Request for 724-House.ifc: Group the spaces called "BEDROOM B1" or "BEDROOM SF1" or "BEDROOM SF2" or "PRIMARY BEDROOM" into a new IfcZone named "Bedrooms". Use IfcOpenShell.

First a look at what the model holds.

```python
import ifcopenshell

model = ifcopenshell.open("724-House.ifc")
print(model.schema)
seen = {}
for space in model.by_type("IfcSpace"):
    seen[space.LongName] = seen.get(space.LongName, 0) + 1
for name, count in sorted(seen.items(), key=str):
    print(count, "x", name)
print("zones:", [z.Name for z in model.by_type("IfcZone")][:20])
```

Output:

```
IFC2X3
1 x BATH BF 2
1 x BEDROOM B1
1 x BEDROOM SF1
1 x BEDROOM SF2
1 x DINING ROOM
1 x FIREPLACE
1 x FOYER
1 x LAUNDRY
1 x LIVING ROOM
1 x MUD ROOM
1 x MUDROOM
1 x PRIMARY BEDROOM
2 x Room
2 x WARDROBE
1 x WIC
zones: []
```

```python
import ifcopenshell
import ifcopenshell.api.group
import ifcopenshell.api.root

model = ifcopenshell.open("724-House.ifc")

names = {"BEDROOM B1", "BEDROOM SF1", "BEDROOM SF2", "PRIMARY BEDROOM"}
spaces = [s for s in model.by_type("IfcSpace") if s.LongName in names]

zone = ifcopenshell.api.root.create_entity(model, ifc_class="IfcZone", name="Bedrooms")
ifcopenshell.api.group.assign_group(model, products=spaces, group=zone)
print(len(spaces), "spaces in", zone.Name)

model.write("724-House_v2.ifc")
```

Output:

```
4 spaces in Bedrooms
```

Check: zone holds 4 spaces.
